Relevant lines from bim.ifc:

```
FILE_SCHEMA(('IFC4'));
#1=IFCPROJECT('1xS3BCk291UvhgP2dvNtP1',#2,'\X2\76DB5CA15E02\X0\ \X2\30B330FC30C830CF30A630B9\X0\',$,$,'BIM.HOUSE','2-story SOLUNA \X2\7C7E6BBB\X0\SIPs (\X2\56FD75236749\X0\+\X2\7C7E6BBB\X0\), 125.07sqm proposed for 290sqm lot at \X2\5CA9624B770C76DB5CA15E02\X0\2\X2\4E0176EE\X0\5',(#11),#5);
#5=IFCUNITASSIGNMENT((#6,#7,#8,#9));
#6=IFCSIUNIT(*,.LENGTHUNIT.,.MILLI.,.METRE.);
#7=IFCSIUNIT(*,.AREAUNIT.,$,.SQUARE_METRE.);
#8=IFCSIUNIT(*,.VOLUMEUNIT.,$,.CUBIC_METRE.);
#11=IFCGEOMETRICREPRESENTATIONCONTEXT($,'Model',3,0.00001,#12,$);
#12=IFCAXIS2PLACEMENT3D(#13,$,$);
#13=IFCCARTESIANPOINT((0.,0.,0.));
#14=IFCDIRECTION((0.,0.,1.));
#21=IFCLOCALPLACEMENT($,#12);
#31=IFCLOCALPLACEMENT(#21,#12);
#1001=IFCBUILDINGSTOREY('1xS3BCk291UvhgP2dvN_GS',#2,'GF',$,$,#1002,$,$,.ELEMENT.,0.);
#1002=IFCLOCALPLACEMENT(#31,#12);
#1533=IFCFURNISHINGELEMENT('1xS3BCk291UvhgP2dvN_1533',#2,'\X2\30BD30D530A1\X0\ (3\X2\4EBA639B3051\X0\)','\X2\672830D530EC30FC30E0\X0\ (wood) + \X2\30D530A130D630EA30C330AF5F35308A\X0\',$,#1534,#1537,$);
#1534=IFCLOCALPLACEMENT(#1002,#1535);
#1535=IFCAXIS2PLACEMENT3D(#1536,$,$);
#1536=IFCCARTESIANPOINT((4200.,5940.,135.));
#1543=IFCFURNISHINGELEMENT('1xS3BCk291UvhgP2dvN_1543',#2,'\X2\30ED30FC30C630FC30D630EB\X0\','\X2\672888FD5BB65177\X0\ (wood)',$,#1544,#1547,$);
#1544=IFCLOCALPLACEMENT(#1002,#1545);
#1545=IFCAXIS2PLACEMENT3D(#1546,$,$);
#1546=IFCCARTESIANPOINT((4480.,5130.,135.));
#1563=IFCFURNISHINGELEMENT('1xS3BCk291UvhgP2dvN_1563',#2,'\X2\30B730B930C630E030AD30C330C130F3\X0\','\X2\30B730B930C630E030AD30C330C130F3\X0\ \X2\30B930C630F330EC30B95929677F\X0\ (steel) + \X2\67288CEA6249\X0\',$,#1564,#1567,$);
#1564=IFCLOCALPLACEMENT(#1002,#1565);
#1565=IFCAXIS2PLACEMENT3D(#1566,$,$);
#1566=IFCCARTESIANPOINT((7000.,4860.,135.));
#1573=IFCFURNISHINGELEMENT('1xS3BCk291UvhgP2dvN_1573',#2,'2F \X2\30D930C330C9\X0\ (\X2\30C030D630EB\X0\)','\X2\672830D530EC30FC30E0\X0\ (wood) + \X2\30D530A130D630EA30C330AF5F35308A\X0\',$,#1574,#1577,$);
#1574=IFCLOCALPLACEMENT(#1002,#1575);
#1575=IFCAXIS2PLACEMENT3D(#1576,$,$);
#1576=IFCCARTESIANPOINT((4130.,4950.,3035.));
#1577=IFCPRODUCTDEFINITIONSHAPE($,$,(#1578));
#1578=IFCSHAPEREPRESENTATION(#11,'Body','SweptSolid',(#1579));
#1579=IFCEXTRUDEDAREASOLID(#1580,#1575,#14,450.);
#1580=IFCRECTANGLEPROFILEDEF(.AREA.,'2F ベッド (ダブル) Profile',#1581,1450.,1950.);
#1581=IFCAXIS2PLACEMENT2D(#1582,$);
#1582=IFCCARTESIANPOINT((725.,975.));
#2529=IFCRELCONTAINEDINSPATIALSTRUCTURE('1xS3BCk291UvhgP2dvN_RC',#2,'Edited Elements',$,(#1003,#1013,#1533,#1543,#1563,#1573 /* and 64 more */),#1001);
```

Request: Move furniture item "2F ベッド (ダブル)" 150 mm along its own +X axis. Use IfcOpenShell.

```python
import ifcopenshell
import ifcopenshell.api.geometry
import ifcopenshell.util.placement

model = ifcopenshell.open("bim.ifc")

item = model.by_id(1573)
matrix = ifcopenshell.util.placement.get_local_placement(item.ObjectPlacement)
matrix[:3, 3] += matrix[:3, 0] * 150.0
ifcopenshell.api.geometry.edit_object_placement(model, product=item, matrix=matrix, is_si=False)

print(ifcopenshell.util.placement.get_local_placement(item.ObjectPlacement).round(3) + 0.0)

model.write("bim-out.ifc")
```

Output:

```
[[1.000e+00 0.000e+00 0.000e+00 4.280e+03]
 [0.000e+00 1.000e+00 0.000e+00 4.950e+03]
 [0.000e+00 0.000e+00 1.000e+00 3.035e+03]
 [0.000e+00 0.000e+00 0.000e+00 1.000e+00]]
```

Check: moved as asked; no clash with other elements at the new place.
